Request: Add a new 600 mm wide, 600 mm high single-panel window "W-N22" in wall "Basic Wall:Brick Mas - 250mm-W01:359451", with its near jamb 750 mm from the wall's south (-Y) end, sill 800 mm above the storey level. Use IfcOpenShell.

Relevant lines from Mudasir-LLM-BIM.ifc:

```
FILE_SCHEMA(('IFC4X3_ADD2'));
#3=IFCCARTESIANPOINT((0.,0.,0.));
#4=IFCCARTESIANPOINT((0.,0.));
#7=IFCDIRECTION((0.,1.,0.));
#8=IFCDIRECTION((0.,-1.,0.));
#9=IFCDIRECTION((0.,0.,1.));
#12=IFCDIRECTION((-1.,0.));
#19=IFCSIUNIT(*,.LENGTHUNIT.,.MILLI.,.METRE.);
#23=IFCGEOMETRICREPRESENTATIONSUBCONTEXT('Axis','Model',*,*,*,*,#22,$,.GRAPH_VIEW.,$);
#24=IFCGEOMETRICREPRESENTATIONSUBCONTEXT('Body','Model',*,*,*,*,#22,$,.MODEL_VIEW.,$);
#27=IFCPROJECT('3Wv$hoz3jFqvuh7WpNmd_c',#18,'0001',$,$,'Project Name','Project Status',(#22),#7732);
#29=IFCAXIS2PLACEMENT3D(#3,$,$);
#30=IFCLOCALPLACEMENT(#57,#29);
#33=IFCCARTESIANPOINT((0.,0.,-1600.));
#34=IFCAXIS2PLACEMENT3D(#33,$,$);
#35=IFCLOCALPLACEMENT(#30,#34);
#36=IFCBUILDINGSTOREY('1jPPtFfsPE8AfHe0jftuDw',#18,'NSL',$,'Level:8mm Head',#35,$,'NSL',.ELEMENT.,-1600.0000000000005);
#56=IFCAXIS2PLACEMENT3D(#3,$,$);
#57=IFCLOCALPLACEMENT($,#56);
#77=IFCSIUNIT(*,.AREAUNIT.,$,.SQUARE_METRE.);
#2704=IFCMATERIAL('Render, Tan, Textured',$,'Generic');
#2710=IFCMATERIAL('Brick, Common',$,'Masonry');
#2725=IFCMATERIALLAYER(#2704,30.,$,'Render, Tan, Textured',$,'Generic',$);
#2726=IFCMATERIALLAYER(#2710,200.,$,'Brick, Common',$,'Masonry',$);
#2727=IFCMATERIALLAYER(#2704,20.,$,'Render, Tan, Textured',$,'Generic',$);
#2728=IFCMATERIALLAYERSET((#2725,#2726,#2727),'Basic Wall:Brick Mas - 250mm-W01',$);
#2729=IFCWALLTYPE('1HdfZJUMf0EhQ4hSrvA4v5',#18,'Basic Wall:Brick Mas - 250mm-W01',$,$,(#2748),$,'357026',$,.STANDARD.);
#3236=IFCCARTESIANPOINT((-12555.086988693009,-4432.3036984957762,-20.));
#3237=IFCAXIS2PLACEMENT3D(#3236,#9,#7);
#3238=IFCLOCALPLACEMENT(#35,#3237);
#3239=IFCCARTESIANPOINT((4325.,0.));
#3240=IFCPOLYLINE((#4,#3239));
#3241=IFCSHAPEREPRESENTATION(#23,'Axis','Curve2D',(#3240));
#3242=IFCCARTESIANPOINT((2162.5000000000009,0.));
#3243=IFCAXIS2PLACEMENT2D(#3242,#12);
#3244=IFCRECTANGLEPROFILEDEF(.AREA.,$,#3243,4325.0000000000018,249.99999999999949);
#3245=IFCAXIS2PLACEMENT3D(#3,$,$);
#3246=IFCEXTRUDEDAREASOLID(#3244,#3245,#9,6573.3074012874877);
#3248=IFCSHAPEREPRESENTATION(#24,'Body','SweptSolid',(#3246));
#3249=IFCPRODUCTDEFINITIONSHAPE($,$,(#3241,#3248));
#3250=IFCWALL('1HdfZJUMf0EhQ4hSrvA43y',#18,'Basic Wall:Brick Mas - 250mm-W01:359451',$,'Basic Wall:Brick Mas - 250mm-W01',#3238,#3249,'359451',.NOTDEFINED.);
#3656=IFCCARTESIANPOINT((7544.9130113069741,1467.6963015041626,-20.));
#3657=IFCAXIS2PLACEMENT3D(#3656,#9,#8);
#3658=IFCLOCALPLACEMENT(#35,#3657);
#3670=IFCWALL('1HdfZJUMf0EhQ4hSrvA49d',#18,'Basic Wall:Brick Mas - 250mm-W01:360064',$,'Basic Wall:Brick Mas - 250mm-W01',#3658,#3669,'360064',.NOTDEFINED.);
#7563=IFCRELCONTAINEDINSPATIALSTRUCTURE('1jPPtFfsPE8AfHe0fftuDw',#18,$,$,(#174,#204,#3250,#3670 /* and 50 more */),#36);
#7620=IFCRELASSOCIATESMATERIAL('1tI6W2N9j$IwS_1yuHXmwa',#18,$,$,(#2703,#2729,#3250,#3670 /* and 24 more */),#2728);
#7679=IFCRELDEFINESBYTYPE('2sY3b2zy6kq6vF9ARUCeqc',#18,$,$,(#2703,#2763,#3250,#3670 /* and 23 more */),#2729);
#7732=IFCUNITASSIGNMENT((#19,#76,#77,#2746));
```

```python
import numpy as np
import ifcopenshell
import ifcopenshell.api.feature
import ifcopenshell.api.geometry
import ifcopenshell.api.root
import ifcopenshell.api.spatial
import ifcopenshell.geom
import ifcopenshell.util.element
import ifcopenshell.util.placement
import ifcopenshell.util.representation
import ifcopenshell.util.shape
import ifcopenshell.util.unit

model = ifcopenshell.open("Mudasir-LLM-BIM.ifc")
unit_scale = ifcopenshell.util.unit.calculate_unit_scale(model)
settings = ifcopenshell.geom.settings()


def volume(element):
    """Net volume in cubic metres, openings subtracted."""
    shape = ifcopenshell.geom.create_shape(settings, element)
    return ifcopenshell.util.shape.get_volume(shape.geometry)


wall = model.by_guid("1HdfZJUMf0EhQ4hSrvA43y")
storey = ifcopenshell.util.element.get_container(wall, ifc_class="IfcBuildingStorey")
context = ifcopenshell.util.representation.get_context(model, "Model", "Body", "MODEL_VIEW")
before = volume(wall)

width, height, from_end, sill = 0.6, 0.6, 0.75, 0.8  # metres

# The wall runs along its own X axis, and the end named is its -X end.
wall_shape = ifcopenshell.geom.create_shape(settings, wall)
x, y, z = ifcopenshell.util.shape.get_vertices(wall_shape.geometry).T
start = x.min() + from_end
face, thickness = float(y.min()), float(y.max() - y.min())
wall_matrix = ifcopenshell.util.placement.get_local_placement(wall.ObjectPlacement)
level = ifcopenshell.util.placement.get_local_placement(storey.ObjectPlacement)[2, 3]


def in_wall(x, y):
    """Placement at x, y metres in the wall's axes, at sill height."""
    matrix = wall_matrix.copy()
    matrix[:, 3] = wall_matrix @ np.array([x / unit_scale, y / unit_scale, 0.0, 1.0])
    matrix[2, 3] = level + sill / unit_scale
    return matrix


# Opening: a box that overshoots both wall faces by 50 mm.
opening = ifcopenshell.api.root.create_entity(model, ifc_class="IfcOpeningElement", predefined_type="OPENING")
box = ifcopenshell.api.geometry.add_wall_representation(
    model, context=context, length=width, height=height, thickness=thickness + 0.1
)
ifcopenshell.api.geometry.assign_representation(model, product=opening, representation=box)
ifcopenshell.api.geometry.edit_object_placement(model, product=opening, matrix=in_wall(start, face - 0.05), is_si=False)
ifcopenshell.api.feature.add_feature(model, feature=opening, element=wall)

window = ifcopenshell.api.root.create_entity(model, ifc_class="IfcWindow", name="W-N22", predefined_type="WINDOW")
window.OverallWidth, window.OverallHeight = width / unit_scale, height / unit_scale
window.PartitioningType = "SINGLE_PANEL"
body = ifcopenshell.api.geometry.add_window_representation(
    model,
    context=context,
    overall_width=window.OverallWidth,
    overall_height=window.OverallHeight,
    partition_type="SINGLE_PANEL",
)
ifcopenshell.api.geometry.assign_representation(model, product=window, representation=body)
ifcopenshell.api.spatial.assign_container(model, products=[window], relating_structure=storey)
ifcopenshell.api.feature.add_filling(model, opening=opening, element=window)

# Centre the window in the wall's thickness.
ifcopenshell.api.geometry.edit_object_placement(model, product=window, matrix=in_wall(start, face), is_si=False)
window_shape = ifcopenshell.geom.create_shape(settings, window)
depth = ifcopenshell.util.shape.get_vertices(window_shape.geometry)[:, 1]
offset = face + thickness / 2 - (depth.min() + depth.max()) / 2
ifcopenshell.api.geometry.edit_object_placement(model, product=window, matrix=in_wall(start, offset), is_si=False)

after = volume(wall)

print(f"wall volume {before:.3f} -> {after:.3f} m3")

model.write("Mudasir-LLM-BIM_v2.ifc")
```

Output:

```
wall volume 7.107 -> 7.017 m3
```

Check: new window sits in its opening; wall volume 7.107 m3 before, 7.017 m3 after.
